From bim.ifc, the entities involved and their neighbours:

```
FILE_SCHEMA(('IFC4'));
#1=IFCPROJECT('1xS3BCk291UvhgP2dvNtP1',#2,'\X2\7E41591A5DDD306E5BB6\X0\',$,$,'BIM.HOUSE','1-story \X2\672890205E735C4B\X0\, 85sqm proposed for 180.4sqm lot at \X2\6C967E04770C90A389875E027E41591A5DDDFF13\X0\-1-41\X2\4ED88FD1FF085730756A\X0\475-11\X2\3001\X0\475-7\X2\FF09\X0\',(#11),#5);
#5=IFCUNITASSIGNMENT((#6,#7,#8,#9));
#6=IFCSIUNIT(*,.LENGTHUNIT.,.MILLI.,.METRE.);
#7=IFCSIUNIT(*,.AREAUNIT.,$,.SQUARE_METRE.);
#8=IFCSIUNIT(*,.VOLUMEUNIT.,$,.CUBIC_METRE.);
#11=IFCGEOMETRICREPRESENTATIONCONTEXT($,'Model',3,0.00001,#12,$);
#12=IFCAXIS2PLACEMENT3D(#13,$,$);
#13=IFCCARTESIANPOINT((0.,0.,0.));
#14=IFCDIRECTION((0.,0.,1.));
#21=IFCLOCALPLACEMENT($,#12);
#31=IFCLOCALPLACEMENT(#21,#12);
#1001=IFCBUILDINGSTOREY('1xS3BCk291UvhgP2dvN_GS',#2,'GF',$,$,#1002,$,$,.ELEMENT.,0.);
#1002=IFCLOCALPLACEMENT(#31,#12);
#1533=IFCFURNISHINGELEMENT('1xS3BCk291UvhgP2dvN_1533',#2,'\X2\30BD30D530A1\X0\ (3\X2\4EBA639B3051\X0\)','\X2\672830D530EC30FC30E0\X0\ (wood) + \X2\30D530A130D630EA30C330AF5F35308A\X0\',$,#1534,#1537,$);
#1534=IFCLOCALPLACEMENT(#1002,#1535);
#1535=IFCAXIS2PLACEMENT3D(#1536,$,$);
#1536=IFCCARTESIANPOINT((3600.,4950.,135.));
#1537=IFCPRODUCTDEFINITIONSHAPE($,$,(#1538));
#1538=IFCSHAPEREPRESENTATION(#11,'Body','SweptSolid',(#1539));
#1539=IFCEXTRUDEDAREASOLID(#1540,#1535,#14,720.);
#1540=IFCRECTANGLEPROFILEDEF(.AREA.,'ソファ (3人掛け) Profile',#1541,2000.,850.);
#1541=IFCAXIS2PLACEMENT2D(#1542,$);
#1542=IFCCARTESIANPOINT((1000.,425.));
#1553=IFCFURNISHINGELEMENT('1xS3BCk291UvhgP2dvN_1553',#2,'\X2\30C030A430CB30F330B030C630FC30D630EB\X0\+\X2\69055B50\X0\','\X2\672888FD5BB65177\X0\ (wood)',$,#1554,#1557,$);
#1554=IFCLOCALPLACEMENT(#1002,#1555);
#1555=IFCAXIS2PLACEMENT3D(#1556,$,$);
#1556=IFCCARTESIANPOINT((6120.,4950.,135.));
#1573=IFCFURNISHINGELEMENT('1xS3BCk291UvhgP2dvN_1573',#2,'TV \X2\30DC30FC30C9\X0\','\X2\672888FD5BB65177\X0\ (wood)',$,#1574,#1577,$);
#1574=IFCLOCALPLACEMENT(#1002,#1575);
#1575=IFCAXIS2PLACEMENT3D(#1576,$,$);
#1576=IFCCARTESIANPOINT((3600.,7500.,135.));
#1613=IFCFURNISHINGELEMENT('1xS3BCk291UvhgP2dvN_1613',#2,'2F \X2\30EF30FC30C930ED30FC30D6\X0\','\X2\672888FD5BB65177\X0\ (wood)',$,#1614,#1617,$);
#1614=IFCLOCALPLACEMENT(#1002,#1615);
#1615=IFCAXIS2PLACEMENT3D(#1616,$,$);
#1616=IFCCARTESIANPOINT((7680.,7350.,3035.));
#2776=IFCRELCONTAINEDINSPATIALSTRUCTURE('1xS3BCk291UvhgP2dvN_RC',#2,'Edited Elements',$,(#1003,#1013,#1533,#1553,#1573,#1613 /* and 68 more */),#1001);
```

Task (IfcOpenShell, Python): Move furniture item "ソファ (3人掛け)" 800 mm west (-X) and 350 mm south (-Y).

```python
import ifcopenshell
import ifcopenshell.api.geometry
import ifcopenshell.util.placement
import ifcopenshell.util.unit

model = ifcopenshell.open("bim.ifc")
unit_scale = ifcopenshell.util.unit.calculate_unit_scale(model)

item = model.by_id(1533)
matrix = ifcopenshell.util.placement.get_local_placement(item.ObjectPlacement)
matrix[0, 3] -= 0.8 / unit_scale
matrix[1, 3] -= 0.35 / unit_scale
ifcopenshell.api.geometry.edit_object_placement(model, product=item, matrix=matrix, is_si=False)

print(ifcopenshell.util.placement.get_local_placement(item.ObjectPlacement).round(3) + 0.0)

model.write("bim_rev.ifc")
```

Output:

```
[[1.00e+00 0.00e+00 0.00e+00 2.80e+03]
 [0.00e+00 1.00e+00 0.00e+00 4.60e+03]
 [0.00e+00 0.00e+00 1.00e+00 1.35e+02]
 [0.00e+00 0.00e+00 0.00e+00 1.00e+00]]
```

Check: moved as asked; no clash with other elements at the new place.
